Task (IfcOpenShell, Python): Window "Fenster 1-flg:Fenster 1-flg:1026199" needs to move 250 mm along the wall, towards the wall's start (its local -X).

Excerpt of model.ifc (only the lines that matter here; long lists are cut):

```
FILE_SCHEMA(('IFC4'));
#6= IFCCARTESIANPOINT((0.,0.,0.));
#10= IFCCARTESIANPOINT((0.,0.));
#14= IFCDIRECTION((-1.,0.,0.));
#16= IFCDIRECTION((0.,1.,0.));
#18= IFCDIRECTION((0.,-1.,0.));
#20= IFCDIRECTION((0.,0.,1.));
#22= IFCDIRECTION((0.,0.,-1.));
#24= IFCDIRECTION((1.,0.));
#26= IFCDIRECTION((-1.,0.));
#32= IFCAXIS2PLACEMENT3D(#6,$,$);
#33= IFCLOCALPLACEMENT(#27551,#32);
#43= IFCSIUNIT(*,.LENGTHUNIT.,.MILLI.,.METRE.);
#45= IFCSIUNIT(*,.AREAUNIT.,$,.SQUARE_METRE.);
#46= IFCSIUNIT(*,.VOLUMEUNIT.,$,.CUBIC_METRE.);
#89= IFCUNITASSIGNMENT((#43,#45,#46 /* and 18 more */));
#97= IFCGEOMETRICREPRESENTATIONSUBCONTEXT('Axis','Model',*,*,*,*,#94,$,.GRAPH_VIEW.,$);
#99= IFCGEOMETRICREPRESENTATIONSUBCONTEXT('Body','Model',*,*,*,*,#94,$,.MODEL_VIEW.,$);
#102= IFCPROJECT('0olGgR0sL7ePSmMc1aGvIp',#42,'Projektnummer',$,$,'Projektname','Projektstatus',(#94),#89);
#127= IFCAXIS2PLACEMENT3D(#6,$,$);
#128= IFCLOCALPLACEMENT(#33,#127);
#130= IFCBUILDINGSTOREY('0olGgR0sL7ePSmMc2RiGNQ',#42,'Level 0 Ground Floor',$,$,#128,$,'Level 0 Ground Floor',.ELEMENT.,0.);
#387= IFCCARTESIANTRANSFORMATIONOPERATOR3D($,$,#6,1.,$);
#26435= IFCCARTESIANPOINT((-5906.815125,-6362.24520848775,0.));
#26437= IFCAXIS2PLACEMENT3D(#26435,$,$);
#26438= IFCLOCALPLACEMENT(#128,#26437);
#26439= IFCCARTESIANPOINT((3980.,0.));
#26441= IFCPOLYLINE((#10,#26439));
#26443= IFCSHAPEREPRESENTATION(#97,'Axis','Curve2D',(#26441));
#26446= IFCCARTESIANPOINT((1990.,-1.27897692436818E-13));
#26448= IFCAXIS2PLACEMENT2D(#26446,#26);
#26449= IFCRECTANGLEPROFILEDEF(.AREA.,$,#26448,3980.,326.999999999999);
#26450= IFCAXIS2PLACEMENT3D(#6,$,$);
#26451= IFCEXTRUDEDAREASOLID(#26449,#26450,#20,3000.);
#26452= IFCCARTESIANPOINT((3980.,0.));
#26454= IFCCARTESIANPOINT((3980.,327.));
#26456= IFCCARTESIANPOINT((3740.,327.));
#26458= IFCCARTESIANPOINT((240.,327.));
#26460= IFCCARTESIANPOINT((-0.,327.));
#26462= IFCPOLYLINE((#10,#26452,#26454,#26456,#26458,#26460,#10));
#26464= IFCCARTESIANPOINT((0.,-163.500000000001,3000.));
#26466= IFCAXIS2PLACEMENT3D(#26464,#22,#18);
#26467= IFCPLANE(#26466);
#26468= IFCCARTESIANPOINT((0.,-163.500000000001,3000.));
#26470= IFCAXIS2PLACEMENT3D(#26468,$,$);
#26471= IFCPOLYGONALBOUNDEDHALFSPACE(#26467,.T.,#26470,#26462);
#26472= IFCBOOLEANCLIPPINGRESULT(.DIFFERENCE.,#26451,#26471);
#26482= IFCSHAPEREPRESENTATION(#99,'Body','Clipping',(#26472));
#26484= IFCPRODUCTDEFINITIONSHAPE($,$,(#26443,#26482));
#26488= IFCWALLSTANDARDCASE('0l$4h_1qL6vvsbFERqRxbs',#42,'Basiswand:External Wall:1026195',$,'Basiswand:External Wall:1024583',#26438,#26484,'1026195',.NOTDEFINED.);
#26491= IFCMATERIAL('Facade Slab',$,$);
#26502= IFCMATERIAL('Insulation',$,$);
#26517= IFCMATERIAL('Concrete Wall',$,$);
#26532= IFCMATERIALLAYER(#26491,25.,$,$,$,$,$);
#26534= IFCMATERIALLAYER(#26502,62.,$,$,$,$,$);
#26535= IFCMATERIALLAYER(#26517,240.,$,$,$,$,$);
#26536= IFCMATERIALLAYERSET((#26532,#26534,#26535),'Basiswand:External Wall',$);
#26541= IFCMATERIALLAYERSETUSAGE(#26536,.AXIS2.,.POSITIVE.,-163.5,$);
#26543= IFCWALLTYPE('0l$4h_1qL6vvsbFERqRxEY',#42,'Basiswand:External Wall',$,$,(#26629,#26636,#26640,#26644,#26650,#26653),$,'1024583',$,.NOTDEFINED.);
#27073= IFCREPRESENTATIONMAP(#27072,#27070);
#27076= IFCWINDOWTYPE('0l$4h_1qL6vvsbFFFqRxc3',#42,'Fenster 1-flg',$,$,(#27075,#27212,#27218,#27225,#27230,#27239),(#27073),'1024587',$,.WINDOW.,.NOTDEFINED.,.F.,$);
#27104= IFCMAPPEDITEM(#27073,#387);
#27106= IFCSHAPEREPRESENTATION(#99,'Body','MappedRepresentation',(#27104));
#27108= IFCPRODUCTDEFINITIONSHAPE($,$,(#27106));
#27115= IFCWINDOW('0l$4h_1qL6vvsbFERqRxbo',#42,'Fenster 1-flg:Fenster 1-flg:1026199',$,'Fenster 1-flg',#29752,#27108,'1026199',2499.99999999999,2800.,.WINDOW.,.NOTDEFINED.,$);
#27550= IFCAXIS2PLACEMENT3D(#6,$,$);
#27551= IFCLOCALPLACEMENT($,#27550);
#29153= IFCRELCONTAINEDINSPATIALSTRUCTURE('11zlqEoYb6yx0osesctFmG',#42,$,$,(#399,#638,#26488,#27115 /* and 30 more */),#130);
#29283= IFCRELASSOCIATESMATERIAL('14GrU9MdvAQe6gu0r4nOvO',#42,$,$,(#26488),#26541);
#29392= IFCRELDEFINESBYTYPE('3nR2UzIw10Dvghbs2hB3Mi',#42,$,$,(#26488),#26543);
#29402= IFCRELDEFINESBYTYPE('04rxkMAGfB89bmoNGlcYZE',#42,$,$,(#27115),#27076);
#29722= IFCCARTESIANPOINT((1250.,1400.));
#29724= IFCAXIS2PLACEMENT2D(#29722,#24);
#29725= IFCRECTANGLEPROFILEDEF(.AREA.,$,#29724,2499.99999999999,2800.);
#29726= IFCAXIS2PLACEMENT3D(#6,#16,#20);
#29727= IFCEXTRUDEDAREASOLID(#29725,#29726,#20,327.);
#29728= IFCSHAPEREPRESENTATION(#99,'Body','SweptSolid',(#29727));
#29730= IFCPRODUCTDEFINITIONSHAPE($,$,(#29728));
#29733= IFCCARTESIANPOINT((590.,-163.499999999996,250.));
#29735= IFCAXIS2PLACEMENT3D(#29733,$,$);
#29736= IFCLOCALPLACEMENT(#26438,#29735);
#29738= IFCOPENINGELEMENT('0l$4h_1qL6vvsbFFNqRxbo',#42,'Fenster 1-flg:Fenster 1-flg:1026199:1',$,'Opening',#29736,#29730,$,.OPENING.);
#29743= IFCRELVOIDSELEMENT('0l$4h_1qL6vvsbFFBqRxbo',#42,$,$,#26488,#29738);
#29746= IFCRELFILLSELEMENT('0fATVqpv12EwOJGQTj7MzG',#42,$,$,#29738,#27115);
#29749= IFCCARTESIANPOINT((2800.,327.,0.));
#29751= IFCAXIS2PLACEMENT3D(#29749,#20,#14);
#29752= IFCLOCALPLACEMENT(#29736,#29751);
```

```python
import ifcopenshell
import ifcopenshell.api.geometry
import ifcopenshell.util.placement

model = ifcopenshell.open("model.ifc")

window = model.by_guid("0l$4h_1qL6vvsbFERqRxbo")
opening = window.FillsVoids[0].RelatingOpeningElement
wall = opening.VoidsElements[0].RelatingBuildingElement

wall_matrix = ifcopenshell.util.placement.get_local_placement(wall.ObjectPlacement)
shift = wall_matrix[:3, 0] * -250.0
before = ifcopenshell.util.placement.get_local_placement(window.ObjectPlacement)[:3, 3].copy()

# The window is placed relative to its opening, so it follows when the opening moves.
matrix = ifcopenshell.util.placement.get_local_placement(opening.ObjectPlacement)
matrix[:3, 3] += shift
ifcopenshell.api.geometry.edit_object_placement(
    model, product=opening, matrix=matrix, is_si=False, should_transform_children=True
)

after = ifcopenshell.util.placement.get_local_placement(window.ObjectPlacement)[:3, 3]
print("window moved by", (after - before).round(3) + 0.0)

model.write("model-out.ifc")
```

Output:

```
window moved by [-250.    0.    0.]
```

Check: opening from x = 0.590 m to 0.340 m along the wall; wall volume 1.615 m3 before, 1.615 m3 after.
